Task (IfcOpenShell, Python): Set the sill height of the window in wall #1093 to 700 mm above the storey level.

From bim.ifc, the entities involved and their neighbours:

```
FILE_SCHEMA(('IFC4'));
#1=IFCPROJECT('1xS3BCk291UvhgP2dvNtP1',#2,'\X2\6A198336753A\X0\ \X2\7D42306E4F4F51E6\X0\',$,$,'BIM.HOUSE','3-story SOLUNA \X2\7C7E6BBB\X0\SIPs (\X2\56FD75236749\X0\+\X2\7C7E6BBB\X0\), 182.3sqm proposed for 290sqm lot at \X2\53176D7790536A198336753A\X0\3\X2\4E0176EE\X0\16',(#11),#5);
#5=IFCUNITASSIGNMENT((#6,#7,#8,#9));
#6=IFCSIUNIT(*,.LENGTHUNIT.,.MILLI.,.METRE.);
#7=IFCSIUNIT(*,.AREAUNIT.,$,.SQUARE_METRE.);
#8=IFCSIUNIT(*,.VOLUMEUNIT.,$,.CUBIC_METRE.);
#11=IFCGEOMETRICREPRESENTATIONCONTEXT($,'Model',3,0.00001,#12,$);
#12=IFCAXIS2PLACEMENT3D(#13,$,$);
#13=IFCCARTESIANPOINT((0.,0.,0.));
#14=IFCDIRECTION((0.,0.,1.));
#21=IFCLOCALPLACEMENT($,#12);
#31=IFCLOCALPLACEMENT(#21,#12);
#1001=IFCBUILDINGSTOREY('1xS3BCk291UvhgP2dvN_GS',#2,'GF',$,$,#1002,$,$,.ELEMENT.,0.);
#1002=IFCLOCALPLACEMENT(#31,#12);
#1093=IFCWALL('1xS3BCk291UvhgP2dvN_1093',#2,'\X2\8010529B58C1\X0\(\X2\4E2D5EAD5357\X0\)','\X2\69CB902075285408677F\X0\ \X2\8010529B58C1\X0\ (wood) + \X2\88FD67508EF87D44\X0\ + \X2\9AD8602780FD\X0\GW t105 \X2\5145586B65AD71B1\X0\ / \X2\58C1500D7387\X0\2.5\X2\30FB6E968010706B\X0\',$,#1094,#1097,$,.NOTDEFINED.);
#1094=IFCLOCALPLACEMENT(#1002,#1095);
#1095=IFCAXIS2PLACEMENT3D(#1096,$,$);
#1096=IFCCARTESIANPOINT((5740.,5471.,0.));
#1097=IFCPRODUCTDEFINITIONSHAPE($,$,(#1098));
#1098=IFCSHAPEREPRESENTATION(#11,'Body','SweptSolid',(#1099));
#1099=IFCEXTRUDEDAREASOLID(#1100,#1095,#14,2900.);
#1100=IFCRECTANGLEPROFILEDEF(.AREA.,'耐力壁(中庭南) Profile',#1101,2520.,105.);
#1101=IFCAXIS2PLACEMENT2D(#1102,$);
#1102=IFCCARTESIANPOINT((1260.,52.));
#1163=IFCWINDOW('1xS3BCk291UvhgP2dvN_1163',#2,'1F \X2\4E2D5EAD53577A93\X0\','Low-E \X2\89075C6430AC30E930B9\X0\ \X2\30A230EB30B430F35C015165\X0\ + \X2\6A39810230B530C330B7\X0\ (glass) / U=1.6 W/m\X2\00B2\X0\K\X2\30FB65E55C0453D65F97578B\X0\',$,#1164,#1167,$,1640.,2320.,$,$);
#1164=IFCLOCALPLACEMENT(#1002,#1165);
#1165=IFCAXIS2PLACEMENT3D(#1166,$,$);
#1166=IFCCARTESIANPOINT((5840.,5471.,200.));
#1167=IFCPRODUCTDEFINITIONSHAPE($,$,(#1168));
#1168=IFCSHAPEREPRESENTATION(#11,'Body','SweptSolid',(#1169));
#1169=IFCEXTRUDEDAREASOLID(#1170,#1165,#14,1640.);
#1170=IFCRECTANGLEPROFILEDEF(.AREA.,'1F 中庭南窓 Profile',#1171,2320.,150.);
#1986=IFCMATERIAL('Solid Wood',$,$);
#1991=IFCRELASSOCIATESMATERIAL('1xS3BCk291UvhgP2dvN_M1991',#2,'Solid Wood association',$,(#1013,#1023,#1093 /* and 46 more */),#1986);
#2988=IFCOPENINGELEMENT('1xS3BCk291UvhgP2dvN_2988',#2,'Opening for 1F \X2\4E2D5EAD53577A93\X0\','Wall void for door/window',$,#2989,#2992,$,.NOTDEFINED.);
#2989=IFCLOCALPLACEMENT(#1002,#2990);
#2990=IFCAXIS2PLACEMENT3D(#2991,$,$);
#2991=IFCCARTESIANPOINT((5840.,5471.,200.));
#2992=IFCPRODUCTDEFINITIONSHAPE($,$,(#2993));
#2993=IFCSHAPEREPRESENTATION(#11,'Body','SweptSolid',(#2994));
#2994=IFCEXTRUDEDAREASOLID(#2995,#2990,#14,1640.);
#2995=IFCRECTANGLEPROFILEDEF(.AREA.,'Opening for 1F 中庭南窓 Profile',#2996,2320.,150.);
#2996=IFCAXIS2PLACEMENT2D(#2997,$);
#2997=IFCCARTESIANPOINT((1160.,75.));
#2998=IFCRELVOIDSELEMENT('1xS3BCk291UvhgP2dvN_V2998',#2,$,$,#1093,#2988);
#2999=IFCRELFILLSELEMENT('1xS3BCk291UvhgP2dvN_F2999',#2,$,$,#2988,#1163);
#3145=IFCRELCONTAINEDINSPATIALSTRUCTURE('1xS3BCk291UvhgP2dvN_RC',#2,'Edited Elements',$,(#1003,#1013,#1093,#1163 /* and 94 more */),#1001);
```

```python
import numpy as np
import ifcopenshell
import ifcopenshell.api.geometry
import ifcopenshell.geom
import ifcopenshell.util.element
import ifcopenshell.util.placement
import ifcopenshell.util.shape
import ifcopenshell.util.unit

model = ifcopenshell.open("bim.ifc")
unit_scale = ifcopenshell.util.unit.calculate_unit_scale(model)

window = model.by_guid("1xS3BCk291UvhgP2dvN_1163")
opening = window.FillsVoids[0].RelatingOpeningElement
storey = ifcopenshell.util.element.get_container(window, ifc_class="IfcBuildingStorey")
level = ifcopenshell.util.placement.get_local_placement(storey.ObjectPlacement)[2, 3]

# The opening's origin need not be at the sill, so measure its lowest point.
shape = ifcopenshell.geom.create_shape(ifcopenshell.geom.settings(), opening)
bottom = ifcopenshell.util.shape.get_shape_bottom_elevation(shape, shape.geometry) / unit_scale
dz = level + 0.7 / unit_scale - bottom

shift = np.array([0.0, 0.0, dz])
# The window is not placed relative to its opening, so move both.
for product in (opening, window):
    matrix = ifcopenshell.util.placement.get_local_placement(product.ObjectPlacement)
    matrix[:3, 3] += shift
    ifcopenshell.api.geometry.edit_object_placement(model, product=product, matrix=matrix, is_si=False)

print(f"moved by {dz * unit_scale:+.3f} m")

model.write("bim-out.ifc")
```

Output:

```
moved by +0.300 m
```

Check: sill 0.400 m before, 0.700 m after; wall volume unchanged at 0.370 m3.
